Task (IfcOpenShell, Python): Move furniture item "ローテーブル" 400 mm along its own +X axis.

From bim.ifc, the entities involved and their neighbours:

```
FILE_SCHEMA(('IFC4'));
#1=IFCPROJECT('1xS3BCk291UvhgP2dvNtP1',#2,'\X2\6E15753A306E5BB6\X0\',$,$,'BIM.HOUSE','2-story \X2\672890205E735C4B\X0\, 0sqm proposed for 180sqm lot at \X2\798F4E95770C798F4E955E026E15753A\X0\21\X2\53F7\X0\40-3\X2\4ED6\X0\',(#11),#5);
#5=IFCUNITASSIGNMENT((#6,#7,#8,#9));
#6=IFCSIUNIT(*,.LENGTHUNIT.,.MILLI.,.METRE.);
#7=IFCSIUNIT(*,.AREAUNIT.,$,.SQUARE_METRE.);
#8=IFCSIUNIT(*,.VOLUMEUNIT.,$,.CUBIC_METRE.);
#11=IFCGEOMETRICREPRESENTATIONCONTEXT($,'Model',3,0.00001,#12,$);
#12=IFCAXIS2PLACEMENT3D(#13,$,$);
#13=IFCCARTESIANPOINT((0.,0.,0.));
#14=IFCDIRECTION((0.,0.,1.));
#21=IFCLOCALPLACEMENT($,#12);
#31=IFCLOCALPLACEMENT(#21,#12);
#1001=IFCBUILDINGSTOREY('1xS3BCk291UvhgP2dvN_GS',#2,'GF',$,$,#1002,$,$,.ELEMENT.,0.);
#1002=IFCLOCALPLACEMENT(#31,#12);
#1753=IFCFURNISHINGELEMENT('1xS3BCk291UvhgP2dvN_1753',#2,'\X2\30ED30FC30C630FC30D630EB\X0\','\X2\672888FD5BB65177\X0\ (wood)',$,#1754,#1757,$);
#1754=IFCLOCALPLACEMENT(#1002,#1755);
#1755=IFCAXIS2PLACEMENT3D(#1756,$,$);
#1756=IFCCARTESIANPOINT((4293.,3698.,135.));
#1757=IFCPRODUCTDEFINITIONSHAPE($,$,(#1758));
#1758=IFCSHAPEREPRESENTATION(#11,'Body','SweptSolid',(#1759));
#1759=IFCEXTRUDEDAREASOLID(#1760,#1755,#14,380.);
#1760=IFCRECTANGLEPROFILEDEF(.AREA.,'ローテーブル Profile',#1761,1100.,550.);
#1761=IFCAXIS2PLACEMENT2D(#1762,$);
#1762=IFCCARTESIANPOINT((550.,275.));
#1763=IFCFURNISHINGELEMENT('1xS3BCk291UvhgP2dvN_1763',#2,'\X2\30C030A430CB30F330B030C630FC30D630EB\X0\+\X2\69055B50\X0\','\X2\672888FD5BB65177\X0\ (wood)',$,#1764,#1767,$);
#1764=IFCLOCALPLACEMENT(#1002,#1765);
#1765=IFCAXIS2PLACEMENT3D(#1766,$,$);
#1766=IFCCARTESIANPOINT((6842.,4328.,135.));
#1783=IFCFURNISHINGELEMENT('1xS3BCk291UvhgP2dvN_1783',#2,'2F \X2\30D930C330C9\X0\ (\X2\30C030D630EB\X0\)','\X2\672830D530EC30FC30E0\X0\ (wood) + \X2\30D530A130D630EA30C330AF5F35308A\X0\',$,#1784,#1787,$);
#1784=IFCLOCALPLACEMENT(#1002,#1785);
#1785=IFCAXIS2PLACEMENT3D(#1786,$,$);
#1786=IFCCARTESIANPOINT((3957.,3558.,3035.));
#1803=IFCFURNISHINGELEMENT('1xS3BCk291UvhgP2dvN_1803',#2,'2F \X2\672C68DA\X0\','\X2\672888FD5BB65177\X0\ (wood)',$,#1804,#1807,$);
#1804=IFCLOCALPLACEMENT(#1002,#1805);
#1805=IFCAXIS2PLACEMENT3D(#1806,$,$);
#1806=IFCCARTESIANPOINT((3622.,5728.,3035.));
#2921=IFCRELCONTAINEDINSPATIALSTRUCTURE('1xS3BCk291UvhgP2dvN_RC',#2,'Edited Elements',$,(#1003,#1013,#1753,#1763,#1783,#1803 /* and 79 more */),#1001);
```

```python
import ifcopenshell
import ifcopenshell.api.geometry
import ifcopenshell.util.placement

model = ifcopenshell.open("bim.ifc")

item = model.by_guid("1xS3BCk291UvhgP2dvN_1753")
matrix = ifcopenshell.util.placement.get_local_placement(item.ObjectPlacement)
matrix[:3, 3] += matrix[:3, 0] * 400.0
ifcopenshell.api.geometry.edit_object_placement(model, product=item, matrix=matrix, is_si=False)

print(ifcopenshell.util.placement.get_local_placement(item.ObjectPlacement).round(3) + 0.0)

model.write("bim_rev.ifc")
```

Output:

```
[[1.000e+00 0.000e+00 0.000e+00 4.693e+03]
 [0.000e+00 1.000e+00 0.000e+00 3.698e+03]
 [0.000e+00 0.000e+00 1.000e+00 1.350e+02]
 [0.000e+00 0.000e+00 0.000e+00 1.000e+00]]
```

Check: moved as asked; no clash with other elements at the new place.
